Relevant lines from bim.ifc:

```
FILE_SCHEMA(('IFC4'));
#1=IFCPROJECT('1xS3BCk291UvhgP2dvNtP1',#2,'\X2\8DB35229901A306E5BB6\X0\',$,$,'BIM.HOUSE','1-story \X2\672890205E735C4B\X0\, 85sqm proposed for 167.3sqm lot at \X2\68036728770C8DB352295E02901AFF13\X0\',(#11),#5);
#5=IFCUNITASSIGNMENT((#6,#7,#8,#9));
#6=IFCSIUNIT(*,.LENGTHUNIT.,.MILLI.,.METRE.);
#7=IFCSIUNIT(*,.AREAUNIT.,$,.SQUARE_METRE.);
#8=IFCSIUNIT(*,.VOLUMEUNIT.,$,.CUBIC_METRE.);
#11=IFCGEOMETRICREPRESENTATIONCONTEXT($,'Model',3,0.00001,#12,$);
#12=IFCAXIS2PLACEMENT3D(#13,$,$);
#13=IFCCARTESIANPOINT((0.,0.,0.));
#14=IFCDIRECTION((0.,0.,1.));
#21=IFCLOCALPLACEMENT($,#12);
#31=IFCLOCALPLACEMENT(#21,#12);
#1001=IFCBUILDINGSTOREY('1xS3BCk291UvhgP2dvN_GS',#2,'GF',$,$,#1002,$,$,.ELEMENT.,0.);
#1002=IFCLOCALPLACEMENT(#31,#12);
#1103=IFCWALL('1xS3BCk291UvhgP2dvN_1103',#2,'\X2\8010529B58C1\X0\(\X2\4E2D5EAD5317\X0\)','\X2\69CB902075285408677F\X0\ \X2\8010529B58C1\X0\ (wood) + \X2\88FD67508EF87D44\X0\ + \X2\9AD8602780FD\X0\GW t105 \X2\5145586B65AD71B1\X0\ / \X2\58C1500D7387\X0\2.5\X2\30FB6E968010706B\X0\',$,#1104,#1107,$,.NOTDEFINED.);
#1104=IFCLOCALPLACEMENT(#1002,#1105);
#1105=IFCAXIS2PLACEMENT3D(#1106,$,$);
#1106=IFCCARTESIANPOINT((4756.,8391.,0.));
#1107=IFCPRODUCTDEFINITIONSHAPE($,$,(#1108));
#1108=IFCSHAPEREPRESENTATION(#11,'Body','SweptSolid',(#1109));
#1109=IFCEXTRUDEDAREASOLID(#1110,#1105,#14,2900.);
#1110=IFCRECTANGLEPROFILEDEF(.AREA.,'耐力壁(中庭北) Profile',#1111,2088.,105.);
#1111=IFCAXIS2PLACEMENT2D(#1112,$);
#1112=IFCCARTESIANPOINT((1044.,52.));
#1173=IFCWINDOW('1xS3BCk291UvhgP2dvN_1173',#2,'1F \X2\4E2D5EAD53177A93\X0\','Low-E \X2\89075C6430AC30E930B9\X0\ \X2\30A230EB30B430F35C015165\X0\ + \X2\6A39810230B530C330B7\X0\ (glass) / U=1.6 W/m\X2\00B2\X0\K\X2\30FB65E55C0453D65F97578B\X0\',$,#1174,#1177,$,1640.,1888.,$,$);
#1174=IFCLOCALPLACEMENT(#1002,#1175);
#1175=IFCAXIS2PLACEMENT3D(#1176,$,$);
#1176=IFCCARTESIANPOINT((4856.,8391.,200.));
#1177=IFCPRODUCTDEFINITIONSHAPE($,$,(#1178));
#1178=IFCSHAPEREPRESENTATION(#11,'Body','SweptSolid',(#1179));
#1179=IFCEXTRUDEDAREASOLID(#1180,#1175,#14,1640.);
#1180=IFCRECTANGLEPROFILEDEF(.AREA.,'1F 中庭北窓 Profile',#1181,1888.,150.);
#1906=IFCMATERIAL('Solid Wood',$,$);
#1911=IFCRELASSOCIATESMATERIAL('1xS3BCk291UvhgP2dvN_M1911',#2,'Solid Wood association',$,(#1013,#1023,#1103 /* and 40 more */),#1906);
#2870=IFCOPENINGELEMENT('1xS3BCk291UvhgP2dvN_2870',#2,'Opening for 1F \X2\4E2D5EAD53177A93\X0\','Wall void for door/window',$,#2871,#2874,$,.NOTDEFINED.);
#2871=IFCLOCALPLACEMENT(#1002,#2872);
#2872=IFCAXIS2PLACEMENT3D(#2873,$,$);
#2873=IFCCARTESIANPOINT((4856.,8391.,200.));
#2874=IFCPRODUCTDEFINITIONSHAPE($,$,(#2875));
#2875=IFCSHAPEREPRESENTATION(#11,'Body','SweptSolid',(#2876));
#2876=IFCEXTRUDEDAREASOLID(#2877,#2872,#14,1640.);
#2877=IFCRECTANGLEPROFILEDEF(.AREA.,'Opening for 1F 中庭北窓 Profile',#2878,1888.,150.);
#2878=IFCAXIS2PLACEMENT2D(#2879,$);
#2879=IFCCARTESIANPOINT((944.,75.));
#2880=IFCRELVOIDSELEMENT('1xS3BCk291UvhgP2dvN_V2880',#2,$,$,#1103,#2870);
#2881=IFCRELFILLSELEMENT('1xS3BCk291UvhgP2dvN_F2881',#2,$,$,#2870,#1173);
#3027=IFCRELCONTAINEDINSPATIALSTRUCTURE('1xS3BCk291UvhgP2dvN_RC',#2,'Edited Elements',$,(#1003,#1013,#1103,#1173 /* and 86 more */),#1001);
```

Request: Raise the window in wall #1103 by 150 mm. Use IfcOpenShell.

```python
import numpy as np
import ifcopenshell
import ifcopenshell.api.geometry
import ifcopenshell.util.placement
import ifcopenshell.util.unit

model = ifcopenshell.open("bim.ifc")
unit_scale = ifcopenshell.util.unit.calculate_unit_scale(model)

window = model.by_guid("1xS3BCk291UvhgP2dvN_1173")
opening = window.FillsVoids[0].RelatingOpeningElement
dz = 0.15 / unit_scale

shift = np.array([0.0, 0.0, dz])
# The window is not placed relative to its opening, so move both.
for product in (opening, window):
    matrix = ifcopenshell.util.placement.get_local_placement(product.ObjectPlacement)
    matrix[:3, 3] += shift
    ifcopenshell.api.geometry.edit_object_placement(model, product=product, matrix=matrix, is_si=False)

print(f"moved by {dz * unit_scale:+.3f} m")

model.write("bim_edited.ifc")
```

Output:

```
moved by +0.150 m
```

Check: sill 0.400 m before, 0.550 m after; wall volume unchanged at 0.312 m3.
